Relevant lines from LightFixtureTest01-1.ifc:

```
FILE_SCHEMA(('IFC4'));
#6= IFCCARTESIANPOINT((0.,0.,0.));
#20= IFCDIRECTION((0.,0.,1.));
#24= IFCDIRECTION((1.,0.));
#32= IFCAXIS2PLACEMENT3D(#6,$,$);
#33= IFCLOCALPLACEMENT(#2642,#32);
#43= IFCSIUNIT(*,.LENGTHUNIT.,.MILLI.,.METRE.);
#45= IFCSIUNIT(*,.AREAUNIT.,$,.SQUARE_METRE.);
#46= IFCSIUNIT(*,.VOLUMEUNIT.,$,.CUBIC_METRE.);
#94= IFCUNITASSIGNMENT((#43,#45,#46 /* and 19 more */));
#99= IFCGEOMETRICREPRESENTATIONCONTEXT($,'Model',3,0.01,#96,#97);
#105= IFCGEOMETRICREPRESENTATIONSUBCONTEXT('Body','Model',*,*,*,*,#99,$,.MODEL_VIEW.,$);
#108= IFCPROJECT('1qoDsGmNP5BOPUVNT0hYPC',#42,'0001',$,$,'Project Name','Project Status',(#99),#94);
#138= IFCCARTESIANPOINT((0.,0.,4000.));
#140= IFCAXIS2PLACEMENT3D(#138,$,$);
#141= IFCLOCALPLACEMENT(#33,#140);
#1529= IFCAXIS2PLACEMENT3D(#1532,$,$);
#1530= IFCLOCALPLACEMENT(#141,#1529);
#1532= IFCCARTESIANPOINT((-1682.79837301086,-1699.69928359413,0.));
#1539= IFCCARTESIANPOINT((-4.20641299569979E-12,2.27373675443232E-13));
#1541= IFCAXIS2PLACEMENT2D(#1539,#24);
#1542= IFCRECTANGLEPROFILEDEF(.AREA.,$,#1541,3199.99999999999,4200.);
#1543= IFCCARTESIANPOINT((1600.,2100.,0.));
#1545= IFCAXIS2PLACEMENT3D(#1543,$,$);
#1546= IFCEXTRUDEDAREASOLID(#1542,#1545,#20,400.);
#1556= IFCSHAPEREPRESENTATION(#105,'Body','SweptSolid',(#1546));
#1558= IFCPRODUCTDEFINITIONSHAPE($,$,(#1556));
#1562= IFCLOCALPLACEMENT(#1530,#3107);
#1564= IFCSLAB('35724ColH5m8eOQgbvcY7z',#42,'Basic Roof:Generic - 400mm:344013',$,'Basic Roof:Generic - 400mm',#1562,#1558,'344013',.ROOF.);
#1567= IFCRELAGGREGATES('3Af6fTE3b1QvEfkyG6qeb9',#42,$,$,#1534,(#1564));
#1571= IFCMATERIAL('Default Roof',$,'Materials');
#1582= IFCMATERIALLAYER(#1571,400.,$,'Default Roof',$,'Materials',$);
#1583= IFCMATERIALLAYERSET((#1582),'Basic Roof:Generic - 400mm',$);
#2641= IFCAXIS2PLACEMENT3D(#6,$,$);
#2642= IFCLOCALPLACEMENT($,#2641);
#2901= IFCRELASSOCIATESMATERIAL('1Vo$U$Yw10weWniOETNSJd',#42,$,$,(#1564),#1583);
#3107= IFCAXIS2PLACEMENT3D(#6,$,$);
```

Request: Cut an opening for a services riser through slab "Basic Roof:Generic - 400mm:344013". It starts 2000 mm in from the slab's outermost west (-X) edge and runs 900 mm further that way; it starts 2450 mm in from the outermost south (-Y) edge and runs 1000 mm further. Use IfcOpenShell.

```python
import numpy as np
import ifcopenshell
import ifcopenshell.api.feature
import ifcopenshell.api.geometry
import ifcopenshell.api.root
import ifcopenshell.geom
import ifcopenshell.util.placement
import ifcopenshell.util.representation
import ifcopenshell.util.shape
import ifcopenshell.util.unit

model = ifcopenshell.open("LightFixtureTest01-1.ifc")
unit_scale = ifcopenshell.util.unit.calculate_unit_scale(model)
settings = ifcopenshell.geom.settings()


def volume(element):
    """Net volume in cubic metres, openings subtracted."""
    shape = ifcopenshell.geom.create_shape(settings, element)
    return ifcopenshell.util.shape.get_volume(shape.geometry)


slab = model.by_guid("35724ColH5m8eOQgbvcY7z")
before = volume(slab)

# Extent in the slab's own axes, in metres. The edges named are its -X and -Y sides.
slab_shape = ifcopenshell.geom.create_shape(settings, slab)
vertices = ifcopenshell.util.shape.get_vertices(slab_shape.geometry)
x_min, y_min, bottom = vertices.min(axis=0)
top = vertices[:, 2].max()

opening = ifcopenshell.api.root.create_entity(model, ifc_class="IfcOpeningElement", name="Services riser opening", predefined_type="OPENING")
context = ifcopenshell.util.representation.get_context(model, "Model", "Body", "MODEL_VIEW")
width, depth = 0.9, 1
outline = [(0.0, 0.0), (width, 0.0), (width, depth), (0.0, depth), (0.0, 0.0)]
# Overshoot both faces by 50 mm so the cut is clean.
shape = ifcopenshell.api.geometry.add_slab_representation(
    model, context=context, depth=top - bottom + 0.1, polyline=outline
)
ifcopenshell.api.geometry.assign_representation(model, product=opening, representation=shape)

matrix = ifcopenshell.util.placement.get_local_placement(slab.ObjectPlacement)
matrix[:, 3] = matrix @ np.append(np.array([x_min + 2, y_min + 2.45, bottom - 0.05]) / unit_scale, 1.0)
ifcopenshell.api.geometry.edit_object_placement(model, product=opening, matrix=matrix, is_si=False)
ifcopenshell.api.feature.add_feature(model, feature=opening, element=slab)

after = volume(slab)

print(f"slab volume {before:.3f} -> {after:.3f} m3")

model.write("LightFixtureTest01-1_edited.ifc")
```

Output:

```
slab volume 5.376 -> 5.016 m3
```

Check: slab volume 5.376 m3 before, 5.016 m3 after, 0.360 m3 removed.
